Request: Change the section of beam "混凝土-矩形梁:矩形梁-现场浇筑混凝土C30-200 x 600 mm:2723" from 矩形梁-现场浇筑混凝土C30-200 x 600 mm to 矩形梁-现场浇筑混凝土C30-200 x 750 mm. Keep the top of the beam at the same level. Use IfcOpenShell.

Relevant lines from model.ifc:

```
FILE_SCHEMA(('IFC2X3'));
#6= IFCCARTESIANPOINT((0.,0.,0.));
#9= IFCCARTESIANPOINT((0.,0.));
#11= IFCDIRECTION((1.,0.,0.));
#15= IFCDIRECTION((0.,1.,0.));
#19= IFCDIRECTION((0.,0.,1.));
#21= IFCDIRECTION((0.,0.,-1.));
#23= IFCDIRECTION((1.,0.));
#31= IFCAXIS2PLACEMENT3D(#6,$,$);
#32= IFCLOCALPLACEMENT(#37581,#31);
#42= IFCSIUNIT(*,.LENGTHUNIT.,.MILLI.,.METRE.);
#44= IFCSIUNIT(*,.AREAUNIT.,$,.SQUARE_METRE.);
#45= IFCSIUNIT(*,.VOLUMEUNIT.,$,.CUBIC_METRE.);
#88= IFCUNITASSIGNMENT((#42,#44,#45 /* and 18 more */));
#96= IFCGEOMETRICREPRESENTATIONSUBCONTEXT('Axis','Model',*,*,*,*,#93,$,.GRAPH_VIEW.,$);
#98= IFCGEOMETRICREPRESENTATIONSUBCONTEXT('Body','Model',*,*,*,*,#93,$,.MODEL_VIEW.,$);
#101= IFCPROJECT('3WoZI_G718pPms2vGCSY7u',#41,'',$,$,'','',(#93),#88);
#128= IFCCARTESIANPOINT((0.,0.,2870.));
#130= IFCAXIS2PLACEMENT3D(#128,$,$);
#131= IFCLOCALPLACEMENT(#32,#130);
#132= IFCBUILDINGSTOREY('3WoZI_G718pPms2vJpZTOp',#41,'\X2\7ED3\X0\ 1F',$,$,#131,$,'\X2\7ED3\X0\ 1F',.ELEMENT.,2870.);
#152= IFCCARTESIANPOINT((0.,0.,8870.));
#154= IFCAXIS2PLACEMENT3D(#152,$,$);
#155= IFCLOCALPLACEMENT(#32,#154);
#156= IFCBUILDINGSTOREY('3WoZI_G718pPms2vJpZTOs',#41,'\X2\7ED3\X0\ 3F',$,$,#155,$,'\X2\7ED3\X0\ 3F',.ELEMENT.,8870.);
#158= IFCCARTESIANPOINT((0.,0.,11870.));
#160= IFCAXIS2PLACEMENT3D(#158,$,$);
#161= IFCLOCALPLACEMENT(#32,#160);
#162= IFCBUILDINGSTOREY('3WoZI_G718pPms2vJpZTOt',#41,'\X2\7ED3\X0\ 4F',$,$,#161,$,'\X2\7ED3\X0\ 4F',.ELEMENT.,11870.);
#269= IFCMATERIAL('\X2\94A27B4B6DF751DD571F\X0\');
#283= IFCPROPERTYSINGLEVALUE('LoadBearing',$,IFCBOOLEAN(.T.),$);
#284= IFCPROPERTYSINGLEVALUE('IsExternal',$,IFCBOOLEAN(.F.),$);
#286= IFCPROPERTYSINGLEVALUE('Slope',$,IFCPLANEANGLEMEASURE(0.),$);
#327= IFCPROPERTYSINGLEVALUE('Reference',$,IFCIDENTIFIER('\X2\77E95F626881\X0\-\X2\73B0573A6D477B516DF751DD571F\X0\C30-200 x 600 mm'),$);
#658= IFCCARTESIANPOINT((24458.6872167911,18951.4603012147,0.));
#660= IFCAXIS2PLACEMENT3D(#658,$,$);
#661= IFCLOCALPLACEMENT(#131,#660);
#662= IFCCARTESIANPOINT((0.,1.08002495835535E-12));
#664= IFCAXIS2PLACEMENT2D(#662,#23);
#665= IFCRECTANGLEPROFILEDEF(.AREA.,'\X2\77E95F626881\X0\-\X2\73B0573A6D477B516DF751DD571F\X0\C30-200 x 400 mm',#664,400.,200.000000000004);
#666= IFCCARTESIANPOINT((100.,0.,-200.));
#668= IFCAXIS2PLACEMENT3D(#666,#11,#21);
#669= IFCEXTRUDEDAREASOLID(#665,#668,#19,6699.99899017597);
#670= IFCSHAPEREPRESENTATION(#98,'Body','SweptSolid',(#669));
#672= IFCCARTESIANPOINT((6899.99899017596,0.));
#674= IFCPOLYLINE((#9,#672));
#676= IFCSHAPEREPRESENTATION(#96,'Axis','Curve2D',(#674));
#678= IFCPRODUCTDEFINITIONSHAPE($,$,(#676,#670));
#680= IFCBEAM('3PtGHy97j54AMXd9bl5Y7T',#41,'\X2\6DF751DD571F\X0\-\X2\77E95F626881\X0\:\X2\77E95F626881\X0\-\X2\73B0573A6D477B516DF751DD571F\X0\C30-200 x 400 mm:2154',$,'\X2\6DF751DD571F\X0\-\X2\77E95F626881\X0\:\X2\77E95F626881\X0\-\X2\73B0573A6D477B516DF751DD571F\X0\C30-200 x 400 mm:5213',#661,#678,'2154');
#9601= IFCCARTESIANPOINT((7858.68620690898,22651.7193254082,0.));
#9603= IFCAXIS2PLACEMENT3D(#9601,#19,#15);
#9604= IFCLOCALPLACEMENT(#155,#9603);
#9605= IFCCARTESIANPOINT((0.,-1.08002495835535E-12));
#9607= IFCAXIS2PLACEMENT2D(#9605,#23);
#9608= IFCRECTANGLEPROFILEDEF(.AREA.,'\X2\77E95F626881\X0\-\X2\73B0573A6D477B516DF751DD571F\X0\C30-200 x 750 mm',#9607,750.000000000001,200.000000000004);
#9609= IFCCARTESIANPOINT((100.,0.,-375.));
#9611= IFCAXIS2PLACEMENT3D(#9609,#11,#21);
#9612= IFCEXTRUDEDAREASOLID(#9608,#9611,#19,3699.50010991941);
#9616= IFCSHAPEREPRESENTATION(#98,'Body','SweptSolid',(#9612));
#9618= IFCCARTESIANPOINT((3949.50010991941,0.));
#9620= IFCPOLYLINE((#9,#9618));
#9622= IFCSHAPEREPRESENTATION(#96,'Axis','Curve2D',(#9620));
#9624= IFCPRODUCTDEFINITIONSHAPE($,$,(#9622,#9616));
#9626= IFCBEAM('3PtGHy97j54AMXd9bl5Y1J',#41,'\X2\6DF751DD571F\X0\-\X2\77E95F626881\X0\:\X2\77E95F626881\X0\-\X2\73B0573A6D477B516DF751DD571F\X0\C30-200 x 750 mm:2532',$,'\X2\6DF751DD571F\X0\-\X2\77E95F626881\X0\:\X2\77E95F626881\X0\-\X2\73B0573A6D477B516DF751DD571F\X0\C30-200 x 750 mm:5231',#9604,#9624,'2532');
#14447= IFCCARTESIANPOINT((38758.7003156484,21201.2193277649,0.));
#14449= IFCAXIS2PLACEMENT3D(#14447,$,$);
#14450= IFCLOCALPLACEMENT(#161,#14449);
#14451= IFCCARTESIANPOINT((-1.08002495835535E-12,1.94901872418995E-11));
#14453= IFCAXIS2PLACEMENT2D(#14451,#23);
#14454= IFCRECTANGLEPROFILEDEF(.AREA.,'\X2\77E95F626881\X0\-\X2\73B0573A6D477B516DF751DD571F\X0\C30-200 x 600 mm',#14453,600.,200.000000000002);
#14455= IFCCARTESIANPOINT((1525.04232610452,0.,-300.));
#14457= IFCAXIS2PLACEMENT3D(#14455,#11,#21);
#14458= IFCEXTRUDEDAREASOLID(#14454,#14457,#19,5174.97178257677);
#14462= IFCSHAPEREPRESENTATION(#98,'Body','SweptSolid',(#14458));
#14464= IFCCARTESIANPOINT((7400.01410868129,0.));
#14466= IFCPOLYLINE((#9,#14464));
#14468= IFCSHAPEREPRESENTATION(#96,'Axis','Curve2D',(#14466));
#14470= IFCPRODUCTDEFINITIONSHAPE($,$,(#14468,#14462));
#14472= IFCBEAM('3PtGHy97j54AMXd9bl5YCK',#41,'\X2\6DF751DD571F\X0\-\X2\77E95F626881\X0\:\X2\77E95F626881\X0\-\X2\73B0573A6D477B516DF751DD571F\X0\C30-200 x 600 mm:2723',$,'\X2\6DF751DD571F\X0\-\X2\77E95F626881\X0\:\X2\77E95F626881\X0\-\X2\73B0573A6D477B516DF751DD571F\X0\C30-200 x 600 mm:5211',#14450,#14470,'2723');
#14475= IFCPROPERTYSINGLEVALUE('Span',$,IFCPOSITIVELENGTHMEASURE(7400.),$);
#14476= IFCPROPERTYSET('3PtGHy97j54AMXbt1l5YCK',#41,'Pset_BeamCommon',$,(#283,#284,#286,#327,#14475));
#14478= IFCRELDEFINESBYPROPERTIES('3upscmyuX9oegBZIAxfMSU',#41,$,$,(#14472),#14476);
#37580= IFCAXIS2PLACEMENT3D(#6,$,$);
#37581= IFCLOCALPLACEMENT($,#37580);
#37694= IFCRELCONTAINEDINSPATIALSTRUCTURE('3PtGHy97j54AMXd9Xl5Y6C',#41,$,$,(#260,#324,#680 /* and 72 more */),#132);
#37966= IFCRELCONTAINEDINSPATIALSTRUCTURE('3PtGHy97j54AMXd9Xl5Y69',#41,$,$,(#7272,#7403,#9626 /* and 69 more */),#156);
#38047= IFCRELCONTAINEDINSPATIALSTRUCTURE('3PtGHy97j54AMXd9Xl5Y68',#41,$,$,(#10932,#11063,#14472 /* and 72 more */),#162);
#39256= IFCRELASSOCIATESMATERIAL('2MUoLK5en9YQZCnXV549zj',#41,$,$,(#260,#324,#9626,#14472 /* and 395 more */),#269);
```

```python
import ifcopenshell
import ifcopenshell.api.pset
import ifcopenshell.util.element
import ifcopenshell.util.representation

model = ifcopenshell.open("model.ifc")

member = model.by_id(14472)
source = next(p for p in model.by_type("IfcRectangleProfileDef") if p.ProfileName == "矩形梁-现场浇筑混凝土C30-200 x 750 mm")

body = ifcopenshell.util.representation.get_representation(member, "Model", "Body")
solid = body.Items[0]
old_profile = solid.SweptArea

# Copy the section's sizes but keep this member's own profile position.
profile = ifcopenshell.util.element.copy(model, source)
# Profiles are centred, so shift by half the change in depth to hold the top.
shift = (old_profile.XDim - profile.XDim) / 2
x, y = old_profile.Position.Location.Coordinates
up = (-1.0, 0.0)  # upwards, in the solid's own plane
location = model.createIfcCartesianPoint((x + up[0] * shift, y + up[1] * shift))
profile.Position = model.createIfcAxis2Placement2D(location, old_profile.Position.RefDirection)
solid.SweptArea = profile
if not model.get_total_inverses(old_profile):
    ifcopenshell.util.element.remove_deep2(model, old_profile)
member.Name = member.Name.replace("矩形梁-现场浇筑混凝土C30-200 x 600 mm", "矩形梁-现场浇筑混凝土C30-200 x 750 mm")
member.ObjectType = member.ObjectType.replace("矩形梁-现场浇筑混凝土C30-200 x 600 mm", "矩形梁-现场浇筑混凝土C30-200 x 750 mm")
pset = model.by_id(ifcopenshell.util.element.get_pset(member, "Pset_BeamCommon", should_inherit=False)["id"])
ifcopenshell.api.pset.edit_pset(model, pset=pset, properties={"Reference": "矩形梁-现场浇筑混凝土C30-200 x 750 mm"})

print(solid.SweptArea)

model.write("model_rev.ifc")
```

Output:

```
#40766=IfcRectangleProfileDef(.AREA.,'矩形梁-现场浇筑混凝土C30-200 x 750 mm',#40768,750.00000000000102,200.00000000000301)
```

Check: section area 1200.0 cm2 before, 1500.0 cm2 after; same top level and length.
